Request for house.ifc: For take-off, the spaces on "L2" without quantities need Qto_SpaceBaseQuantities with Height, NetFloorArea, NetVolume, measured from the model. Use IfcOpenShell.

First a look at what the model holds.

```python
import ifcopenshell
import ifcopenshell.util.element
import ifcopenshell.util.unit

model = ifcopenshell.open("house.ifc")
print(model.schema)
for unit_type in ("LENGTHUNIT", "AREAUNIT", "VOLUMEUNIT"):
    print(unit_type, ifcopenshell.util.unit.calculate_unit_scale(model, unit_type))
storey = next(s for s in model.by_type("IfcBuildingStorey") if s.Name == "L2")
spaces = [e for e in ifcopenshell.util.element.get_decomposition(storey) if e.is_a("IfcSpace")]
for e in sorted(spaces, key=lambda e: e.id()):
    print(e.id(), e.is_a(), e.Name, list(ifcopenshell.util.element.get_psets(e, qtos_only=True)), sep=" | ")
```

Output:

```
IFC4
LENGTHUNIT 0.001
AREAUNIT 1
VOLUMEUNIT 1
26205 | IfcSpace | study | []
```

```python
import ifcopenshell
import ifcopenshell.api.pset
import ifcopenshell.geom
import ifcopenshell.util.element
import ifcopenshell.util.shape
import ifcopenshell.util.unit

model = ifcopenshell.open("house.ifc")
unit_scale = ifcopenshell.util.unit.calculate_unit_scale(model)
area_scale = ifcopenshell.util.unit.calculate_unit_scale(model, "AREAUNIT")
volume_scale = ifcopenshell.util.unit.calculate_unit_scale(model, "VOLUMEUNIT")
settings = ifcopenshell.geom.settings()

storey = next(s for s in model.by_type("IfcBuildingStorey") if s.Name == "L2")
spaces = [e for e in ifcopenshell.util.element.get_decomposition(storey) if e.is_a("IfcSpace")]

for e in sorted(spaces, key=lambda e: e.id()):
    if ifcopenshell.util.element.get_psets(e, qtos_only=True, should_inherit=False):
        continue
    # Geometry comes back in metres, in the element's own axes.
    shape = ifcopenshell.geom.create_shape(settings, e)
    values = {
        "Height": ifcopenshell.util.shape.get_z(shape.geometry) / unit_scale,
        "NetFloorArea": ifcopenshell.util.shape.get_footprint_area(shape.geometry) / area_scale,
        "NetVolume": ifcopenshell.util.shape.get_volume(shape.geometry) / volume_scale,
    }
    qto = ifcopenshell.api.pset.add_qto(model, product=e, name="Qto_SpaceBaseQuantities")
    ifcopenshell.api.pset.edit_qto(model, qto=qto, properties=values)
    print(e.id(), {k: round(v, 3) for k, v in values.items()})

model.write("house_v2.ifc")
```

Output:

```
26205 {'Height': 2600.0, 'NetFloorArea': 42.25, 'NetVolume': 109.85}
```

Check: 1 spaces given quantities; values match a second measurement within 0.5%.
